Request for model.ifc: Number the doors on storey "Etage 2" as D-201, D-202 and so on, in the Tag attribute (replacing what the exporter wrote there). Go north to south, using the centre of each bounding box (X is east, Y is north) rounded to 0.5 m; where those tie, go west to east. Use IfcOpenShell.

First a look at what the model holds.

```python
import ifcopenshell
import ifcopenshell.util.element
import ifcopenshell.util.placement

model = ifcopenshell.open("model.ifc")
print(model.schema)
storey = next(s for s in model.by_type("IfcBuildingStorey") if s.Name == "Etage 2")
doors = [e for e in ifcopenshell.util.element.get_decomposition(storey) if e.is_a("IfcDoor")]
for e in sorted(doors, key=lambda e: e.id()):
    origin = ifcopenshell.util.placement.get_local_placement(e.ObjectPlacement)[:3, 3]
    print(e.id(), e.Tag, e.Name, origin.round(2) + 0.0, sep=" | ")
```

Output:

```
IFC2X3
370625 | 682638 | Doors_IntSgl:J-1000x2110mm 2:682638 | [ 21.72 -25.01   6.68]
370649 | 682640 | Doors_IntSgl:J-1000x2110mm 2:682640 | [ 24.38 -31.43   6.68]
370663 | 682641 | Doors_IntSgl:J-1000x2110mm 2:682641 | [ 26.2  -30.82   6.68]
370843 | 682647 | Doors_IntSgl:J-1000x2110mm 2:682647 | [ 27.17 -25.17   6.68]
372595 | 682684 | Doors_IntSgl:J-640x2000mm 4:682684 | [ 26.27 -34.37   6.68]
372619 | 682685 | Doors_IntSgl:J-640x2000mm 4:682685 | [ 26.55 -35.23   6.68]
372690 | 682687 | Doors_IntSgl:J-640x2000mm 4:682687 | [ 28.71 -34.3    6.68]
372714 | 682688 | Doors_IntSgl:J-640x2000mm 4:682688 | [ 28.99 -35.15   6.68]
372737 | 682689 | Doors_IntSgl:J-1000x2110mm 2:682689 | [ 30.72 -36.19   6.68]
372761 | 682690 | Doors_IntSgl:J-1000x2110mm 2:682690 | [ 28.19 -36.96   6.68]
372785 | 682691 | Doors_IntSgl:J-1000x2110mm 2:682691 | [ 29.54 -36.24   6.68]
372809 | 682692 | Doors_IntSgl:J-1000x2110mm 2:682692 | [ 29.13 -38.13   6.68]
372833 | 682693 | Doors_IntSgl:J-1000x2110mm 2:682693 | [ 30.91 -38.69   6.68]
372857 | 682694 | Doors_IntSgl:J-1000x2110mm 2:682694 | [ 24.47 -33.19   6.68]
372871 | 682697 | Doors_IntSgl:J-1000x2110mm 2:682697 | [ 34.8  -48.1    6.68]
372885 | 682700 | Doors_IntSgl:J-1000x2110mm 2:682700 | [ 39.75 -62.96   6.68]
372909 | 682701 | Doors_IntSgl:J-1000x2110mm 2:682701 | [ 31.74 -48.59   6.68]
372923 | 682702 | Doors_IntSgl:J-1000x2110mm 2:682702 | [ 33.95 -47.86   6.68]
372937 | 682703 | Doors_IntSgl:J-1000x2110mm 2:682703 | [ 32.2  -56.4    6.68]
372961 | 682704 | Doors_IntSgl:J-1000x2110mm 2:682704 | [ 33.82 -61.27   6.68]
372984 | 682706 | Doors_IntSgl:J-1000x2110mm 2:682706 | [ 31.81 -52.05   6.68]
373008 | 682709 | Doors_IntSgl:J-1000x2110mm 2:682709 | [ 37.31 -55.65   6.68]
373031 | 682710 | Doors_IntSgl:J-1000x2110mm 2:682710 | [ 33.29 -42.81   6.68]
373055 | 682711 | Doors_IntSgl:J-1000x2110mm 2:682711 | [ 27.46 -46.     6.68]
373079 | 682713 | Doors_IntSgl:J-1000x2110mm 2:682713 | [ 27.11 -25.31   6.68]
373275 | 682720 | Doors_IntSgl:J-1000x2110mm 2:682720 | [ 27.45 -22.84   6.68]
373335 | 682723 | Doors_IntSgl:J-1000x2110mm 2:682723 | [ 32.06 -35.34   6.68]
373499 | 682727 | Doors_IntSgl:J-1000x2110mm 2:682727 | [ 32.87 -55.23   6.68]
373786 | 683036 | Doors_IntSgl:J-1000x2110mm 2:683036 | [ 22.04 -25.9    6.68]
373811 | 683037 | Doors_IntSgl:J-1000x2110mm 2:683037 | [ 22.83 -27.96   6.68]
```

```python
import ifcopenshell
import ifcopenshell.geom
import ifcopenshell.util.element
import ifcopenshell.util.shape

model = ifcopenshell.open("model.ifc")
settings = ifcopenshell.geom.settings()
settings.set("use-world-coords", True)


def centre(element):
    shape = ifcopenshell.geom.create_shape(settings, element)
    return ifcopenshell.util.shape.get_bbox_centroid(shape.geometry)


storey = next(s for s in model.by_type("IfcBuildingStorey") if s.Name == "Etage 2")
doors = [e for e in ifcopenshell.util.element.get_decomposition(storey) if e.is_a("IfcDoor")]

# Insertion points can sit at a corner or the storey origin, so sort by the geometry (in metres).
centres = {e: centre(e) for e in doors}
doors.sort(key=lambda e: (-round(centres[e][1] / 0.5), centres[e][0]))

for i, e in enumerate(doors, start=1):
    number = f"D-2{i:02d}"
    e.Tag = number
    print(e.id(), number)

model.write("model-out.ifc")
```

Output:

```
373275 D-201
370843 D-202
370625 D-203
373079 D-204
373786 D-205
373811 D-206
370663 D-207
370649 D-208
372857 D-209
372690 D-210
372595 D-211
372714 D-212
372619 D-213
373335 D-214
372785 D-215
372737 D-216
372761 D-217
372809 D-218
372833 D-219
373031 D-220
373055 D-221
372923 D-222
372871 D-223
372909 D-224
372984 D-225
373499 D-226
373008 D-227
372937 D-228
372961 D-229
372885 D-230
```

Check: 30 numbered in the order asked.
